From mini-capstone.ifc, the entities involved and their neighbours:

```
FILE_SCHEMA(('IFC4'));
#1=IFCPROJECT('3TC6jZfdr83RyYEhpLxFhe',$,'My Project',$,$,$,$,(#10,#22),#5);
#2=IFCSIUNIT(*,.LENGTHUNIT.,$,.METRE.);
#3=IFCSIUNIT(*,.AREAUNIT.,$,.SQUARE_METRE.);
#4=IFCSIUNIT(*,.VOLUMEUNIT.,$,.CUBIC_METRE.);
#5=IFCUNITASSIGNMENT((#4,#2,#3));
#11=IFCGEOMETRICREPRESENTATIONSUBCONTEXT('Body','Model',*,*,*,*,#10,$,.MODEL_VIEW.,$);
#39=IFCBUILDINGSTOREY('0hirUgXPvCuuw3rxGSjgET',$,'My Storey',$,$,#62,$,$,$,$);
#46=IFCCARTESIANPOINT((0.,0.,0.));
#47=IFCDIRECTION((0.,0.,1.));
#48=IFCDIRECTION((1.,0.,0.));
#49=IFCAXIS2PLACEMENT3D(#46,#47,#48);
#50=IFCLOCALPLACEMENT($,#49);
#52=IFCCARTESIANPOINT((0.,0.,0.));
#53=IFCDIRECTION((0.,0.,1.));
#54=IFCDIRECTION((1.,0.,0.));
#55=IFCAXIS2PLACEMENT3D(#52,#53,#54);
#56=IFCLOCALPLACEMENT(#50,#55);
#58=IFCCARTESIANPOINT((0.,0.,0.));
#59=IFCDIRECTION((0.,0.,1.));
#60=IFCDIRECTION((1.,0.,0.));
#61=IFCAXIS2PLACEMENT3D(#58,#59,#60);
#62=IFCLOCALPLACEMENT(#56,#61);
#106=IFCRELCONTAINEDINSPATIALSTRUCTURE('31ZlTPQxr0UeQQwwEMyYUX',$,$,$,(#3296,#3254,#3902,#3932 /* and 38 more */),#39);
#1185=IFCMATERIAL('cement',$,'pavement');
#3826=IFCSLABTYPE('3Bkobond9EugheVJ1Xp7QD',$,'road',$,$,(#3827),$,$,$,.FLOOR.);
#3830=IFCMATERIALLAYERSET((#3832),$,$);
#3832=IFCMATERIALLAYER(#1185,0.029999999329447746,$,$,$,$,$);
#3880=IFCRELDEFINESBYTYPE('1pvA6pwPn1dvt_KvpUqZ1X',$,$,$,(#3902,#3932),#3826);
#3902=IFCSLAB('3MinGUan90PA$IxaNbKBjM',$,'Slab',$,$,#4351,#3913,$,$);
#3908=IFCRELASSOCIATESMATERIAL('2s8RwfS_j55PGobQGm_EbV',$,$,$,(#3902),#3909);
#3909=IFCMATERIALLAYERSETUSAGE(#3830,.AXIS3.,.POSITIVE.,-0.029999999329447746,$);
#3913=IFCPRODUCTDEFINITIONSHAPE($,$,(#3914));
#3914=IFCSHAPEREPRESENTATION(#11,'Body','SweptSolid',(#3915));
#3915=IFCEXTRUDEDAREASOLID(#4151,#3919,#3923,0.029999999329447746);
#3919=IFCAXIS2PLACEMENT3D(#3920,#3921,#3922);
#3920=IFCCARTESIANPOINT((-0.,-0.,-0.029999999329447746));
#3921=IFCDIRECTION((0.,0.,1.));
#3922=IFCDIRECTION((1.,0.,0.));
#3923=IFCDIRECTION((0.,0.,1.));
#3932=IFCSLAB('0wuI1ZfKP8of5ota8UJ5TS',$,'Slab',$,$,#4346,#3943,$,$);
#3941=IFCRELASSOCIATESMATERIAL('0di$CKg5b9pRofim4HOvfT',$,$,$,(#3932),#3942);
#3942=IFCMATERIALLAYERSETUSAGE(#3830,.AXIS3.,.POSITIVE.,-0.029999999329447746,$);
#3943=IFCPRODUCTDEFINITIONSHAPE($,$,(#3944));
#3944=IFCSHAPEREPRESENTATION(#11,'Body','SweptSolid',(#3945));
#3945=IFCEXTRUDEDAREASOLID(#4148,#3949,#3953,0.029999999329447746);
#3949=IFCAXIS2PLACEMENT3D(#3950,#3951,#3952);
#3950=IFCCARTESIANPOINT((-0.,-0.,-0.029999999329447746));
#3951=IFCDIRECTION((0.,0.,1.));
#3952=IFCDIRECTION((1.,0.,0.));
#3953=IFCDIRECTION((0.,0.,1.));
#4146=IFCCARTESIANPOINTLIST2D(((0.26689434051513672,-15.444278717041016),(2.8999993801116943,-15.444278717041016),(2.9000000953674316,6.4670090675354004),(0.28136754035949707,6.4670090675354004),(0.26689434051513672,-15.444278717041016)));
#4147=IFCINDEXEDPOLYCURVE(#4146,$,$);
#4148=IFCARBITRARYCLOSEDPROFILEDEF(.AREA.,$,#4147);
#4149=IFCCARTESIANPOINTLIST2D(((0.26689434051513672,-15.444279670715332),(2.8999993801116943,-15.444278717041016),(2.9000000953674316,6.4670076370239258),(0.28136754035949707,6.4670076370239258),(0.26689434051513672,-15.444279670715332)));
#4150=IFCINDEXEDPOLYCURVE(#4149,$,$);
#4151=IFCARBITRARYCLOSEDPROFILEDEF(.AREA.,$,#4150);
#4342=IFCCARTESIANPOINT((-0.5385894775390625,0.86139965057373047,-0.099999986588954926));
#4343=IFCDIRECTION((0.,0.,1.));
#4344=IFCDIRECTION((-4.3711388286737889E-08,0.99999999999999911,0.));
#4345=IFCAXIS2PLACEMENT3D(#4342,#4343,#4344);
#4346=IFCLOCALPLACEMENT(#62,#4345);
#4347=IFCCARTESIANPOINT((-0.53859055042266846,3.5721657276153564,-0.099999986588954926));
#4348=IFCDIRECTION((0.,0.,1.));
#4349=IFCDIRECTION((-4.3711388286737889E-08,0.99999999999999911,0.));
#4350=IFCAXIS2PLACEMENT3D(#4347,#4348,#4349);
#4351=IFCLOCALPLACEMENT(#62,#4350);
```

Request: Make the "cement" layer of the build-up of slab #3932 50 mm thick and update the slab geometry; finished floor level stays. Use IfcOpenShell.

```python
import ifcopenshell
import ifcopenshell.util.element
import ifcopenshell.util.representation
import ifcopenshell.util.unit

model = ifcopenshell.open("mini-capstone.ifc")
unit_scale = ifcopenshell.util.unit.calculate_unit_scale(model)

layer_set = model.by_id(3830)
layer = next(l for l in layer_set.MaterialLayers if l.Material and l.Material.Name == "cement")
change = 0.05 / unit_scale - layer.LayerThickness
layer.LayerThickness += change

# The layer set is shared, so every slab that uses it gets the new thickness.
slabs = [e for e in ifcopenshell.util.element.get_elements_by_material(model, layer_set) if e.is_a("IfcSlab")]
for slab in sorted(slabs, key=lambda e: e.id()):
    body = ifcopenshell.util.representation.get_representation(slab, "Model", "Body")
    solid = body.Items[0]
    old_depth = solid.Depth
    solid.Depth += change
    # Extruded upwards: lower the start of the extrusion so the top stays.
    x, y, z = solid.Position.Location.Coordinates
    solid.Position.Location = model.createIfcCartesianPoint((x, y, z - change))
    print(slab.id(), f"{old_depth:g} -> {solid.Depth:g}")

# The layers are counted up from the underside, which has moved.
for usage in {ifcopenshell.util.element.get_material(slab) for slab in slabs}:
    usage.OffsetFromReferenceLine -= change

model.write("mini-capstone_v2.ifc")
```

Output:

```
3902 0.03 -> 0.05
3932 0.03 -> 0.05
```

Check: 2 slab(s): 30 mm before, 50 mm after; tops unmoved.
